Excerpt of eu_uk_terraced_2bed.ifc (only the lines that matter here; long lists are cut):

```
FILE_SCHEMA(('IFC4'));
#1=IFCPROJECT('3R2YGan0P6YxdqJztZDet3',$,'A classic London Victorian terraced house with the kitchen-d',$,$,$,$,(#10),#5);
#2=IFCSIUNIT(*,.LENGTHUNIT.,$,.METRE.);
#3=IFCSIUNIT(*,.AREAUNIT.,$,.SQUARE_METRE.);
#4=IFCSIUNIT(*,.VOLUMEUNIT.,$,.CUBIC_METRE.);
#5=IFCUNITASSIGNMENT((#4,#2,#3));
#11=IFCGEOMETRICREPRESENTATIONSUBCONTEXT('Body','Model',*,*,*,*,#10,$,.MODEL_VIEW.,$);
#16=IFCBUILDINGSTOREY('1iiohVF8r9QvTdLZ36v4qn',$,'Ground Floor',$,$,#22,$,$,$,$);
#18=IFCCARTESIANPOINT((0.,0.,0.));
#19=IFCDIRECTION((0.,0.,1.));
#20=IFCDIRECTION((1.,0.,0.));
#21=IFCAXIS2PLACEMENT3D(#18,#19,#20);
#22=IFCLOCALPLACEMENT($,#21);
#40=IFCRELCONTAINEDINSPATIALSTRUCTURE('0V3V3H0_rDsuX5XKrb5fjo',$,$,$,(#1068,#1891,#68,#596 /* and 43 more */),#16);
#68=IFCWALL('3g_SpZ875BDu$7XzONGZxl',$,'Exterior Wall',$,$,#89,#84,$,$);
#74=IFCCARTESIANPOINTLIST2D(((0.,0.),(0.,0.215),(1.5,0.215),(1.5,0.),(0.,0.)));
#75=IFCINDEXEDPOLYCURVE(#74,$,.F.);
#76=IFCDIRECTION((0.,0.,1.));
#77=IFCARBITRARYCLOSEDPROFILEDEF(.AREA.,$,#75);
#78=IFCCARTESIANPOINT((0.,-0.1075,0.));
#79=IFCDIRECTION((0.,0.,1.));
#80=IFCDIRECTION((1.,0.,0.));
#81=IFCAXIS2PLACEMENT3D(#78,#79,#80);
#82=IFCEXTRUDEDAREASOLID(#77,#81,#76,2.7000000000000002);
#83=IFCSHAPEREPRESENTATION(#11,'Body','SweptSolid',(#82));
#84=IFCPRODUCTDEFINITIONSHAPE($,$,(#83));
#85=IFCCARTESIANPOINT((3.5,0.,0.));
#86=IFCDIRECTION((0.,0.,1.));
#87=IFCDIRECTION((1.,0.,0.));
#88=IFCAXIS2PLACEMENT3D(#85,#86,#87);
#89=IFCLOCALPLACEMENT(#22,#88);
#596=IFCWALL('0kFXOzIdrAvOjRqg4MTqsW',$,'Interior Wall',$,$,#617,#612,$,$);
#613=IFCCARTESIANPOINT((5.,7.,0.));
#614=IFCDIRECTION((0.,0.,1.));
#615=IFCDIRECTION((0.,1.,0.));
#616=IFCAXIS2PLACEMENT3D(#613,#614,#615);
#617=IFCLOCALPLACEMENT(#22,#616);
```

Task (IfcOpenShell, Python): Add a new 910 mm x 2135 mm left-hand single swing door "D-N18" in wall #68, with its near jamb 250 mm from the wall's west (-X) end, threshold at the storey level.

```python
import numpy as np
import ifcopenshell
import ifcopenshell.api.feature
import ifcopenshell.api.geometry
import ifcopenshell.api.root
import ifcopenshell.api.spatial
import ifcopenshell.geom
import ifcopenshell.util.element
import ifcopenshell.util.placement
import ifcopenshell.util.representation
import ifcopenshell.util.shape
import ifcopenshell.util.unit

model = ifcopenshell.open("eu_uk_terraced_2bed.ifc")
unit_scale = ifcopenshell.util.unit.calculate_unit_scale(model)
settings = ifcopenshell.geom.settings()


def volume(element):
    """Net volume in cubic metres, openings subtracted."""
    shape = ifcopenshell.geom.create_shape(settings, element)
    return ifcopenshell.util.shape.get_volume(shape.geometry)


wall = model.by_id(68)
storey = ifcopenshell.util.element.get_container(wall, ifc_class="IfcBuildingStorey")
context = ifcopenshell.util.representation.get_context(model, "Model", "Body", "MODEL_VIEW")
before = volume(wall)

width, height, from_end, sill = 0.91, 2.135, 0.25, 0.0  # metres

# The wall runs along its own X axis, and the end named is its -X end.
wall_shape = ifcopenshell.geom.create_shape(settings, wall)
x, y, z = ifcopenshell.util.shape.get_vertices(wall_shape.geometry).T
start = x.min() + from_end
face, thickness = float(y.min()), float(y.max() - y.min())
wall_matrix = ifcopenshell.util.placement.get_local_placement(wall.ObjectPlacement)
level = ifcopenshell.util.placement.get_local_placement(storey.ObjectPlacement)[2, 3]


def in_wall(x, y):
    """Placement at x, y metres in the wall's axes, at sill height."""
    matrix = wall_matrix.copy()
    matrix[:, 3] = wall_matrix @ np.array([x / unit_scale, y / unit_scale, 0.0, 1.0])
    matrix[2, 3] = level + sill / unit_scale
    return matrix


# Opening: a box that overshoots both wall faces by 50 mm.
opening = ifcopenshell.api.root.create_entity(model, ifc_class="IfcOpeningElement", predefined_type="OPENING")
box = ifcopenshell.api.geometry.add_wall_representation(
    model, context=context, length=width, height=height, thickness=thickness + 0.1
)
ifcopenshell.api.geometry.assign_representation(model, product=opening, representation=box)
ifcopenshell.api.geometry.edit_object_placement(model, product=opening, matrix=in_wall(start, face - 0.05), is_si=False)
ifcopenshell.api.feature.add_feature(model, feature=opening, element=wall)

door = ifcopenshell.api.root.create_entity(model, ifc_class="IfcDoor", name="D-N18", predefined_type="DOOR")
door.OverallWidth, door.OverallHeight = width / unit_scale, height / unit_scale
door.OperationType = "SINGLE_SWING_LEFT"
body = ifcopenshell.api.geometry.add_door_representation(
    model,
    context=context,
    overall_width=door.OverallWidth,
    overall_height=door.OverallHeight,
    operation_type="SINGLE_SWING_LEFT",
    lining_properties={"LiningDepth": thickness / unit_scale, "ThresholdDepth": thickness / unit_scale},
)
ifcopenshell.api.geometry.assign_representation(model, product=door, representation=body)
ifcopenshell.api.spatial.assign_container(model, products=[door], relating_structure=storey)
ifcopenshell.api.feature.add_filling(model, opening=opening, element=door)

# The lining spans the wall, so the door starts at the wall face.
ifcopenshell.api.geometry.edit_object_placement(model, product=door, matrix=in_wall(start, face), is_si=False)

after = volume(wall)

print(f"wall volume {before:.3f} -> {after:.3f} m3")

model.write("eu_uk_terraced_2bed_edited.ifc")
```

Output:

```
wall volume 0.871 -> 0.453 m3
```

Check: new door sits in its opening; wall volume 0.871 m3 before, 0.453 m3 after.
